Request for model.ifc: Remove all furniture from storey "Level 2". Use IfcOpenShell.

First a look at what the model holds.

```python
import ifcopenshell
import ifcopenshell.util.element

model = ifcopenshell.open("model.ifc")
print(model.schema)
storey = next(s for s in model.by_type("IfcBuildingStorey") if s.Name == "Level 2")
furniture = [e for e in ifcopenshell.util.element.get_decomposition(storey) if e.is_a("IfcFurnishingElement")]
seen = {}
for e in furniture:
    element_type = ifcopenshell.util.element.get_type(e)
    name = element_type.Name if element_type not in (None, e) else None
    seen[name] = seen.get(name, 0) + 1
for name, count in sorted(seen.items(), key=str):
    print(count, "x", name)
```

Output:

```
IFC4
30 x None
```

```python
import ifcopenshell
import ifcopenshell.api.root
import ifcopenshell.util.element

model = ifcopenshell.open("model.ifc")

storey = next(s for s in model.by_type("IfcBuildingStorey") if s.Name == "Level 2")
furniture = [e for e in ifcopenshell.util.element.get_decomposition(storey) if e.is_a("IfcFurnishingElement")]

for e in furniture:
    ifcopenshell.api.root.remove_product(model, product=e)
print(len(furniture), "removed")

model.write("model_edited.ifc")
```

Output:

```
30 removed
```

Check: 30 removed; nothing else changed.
